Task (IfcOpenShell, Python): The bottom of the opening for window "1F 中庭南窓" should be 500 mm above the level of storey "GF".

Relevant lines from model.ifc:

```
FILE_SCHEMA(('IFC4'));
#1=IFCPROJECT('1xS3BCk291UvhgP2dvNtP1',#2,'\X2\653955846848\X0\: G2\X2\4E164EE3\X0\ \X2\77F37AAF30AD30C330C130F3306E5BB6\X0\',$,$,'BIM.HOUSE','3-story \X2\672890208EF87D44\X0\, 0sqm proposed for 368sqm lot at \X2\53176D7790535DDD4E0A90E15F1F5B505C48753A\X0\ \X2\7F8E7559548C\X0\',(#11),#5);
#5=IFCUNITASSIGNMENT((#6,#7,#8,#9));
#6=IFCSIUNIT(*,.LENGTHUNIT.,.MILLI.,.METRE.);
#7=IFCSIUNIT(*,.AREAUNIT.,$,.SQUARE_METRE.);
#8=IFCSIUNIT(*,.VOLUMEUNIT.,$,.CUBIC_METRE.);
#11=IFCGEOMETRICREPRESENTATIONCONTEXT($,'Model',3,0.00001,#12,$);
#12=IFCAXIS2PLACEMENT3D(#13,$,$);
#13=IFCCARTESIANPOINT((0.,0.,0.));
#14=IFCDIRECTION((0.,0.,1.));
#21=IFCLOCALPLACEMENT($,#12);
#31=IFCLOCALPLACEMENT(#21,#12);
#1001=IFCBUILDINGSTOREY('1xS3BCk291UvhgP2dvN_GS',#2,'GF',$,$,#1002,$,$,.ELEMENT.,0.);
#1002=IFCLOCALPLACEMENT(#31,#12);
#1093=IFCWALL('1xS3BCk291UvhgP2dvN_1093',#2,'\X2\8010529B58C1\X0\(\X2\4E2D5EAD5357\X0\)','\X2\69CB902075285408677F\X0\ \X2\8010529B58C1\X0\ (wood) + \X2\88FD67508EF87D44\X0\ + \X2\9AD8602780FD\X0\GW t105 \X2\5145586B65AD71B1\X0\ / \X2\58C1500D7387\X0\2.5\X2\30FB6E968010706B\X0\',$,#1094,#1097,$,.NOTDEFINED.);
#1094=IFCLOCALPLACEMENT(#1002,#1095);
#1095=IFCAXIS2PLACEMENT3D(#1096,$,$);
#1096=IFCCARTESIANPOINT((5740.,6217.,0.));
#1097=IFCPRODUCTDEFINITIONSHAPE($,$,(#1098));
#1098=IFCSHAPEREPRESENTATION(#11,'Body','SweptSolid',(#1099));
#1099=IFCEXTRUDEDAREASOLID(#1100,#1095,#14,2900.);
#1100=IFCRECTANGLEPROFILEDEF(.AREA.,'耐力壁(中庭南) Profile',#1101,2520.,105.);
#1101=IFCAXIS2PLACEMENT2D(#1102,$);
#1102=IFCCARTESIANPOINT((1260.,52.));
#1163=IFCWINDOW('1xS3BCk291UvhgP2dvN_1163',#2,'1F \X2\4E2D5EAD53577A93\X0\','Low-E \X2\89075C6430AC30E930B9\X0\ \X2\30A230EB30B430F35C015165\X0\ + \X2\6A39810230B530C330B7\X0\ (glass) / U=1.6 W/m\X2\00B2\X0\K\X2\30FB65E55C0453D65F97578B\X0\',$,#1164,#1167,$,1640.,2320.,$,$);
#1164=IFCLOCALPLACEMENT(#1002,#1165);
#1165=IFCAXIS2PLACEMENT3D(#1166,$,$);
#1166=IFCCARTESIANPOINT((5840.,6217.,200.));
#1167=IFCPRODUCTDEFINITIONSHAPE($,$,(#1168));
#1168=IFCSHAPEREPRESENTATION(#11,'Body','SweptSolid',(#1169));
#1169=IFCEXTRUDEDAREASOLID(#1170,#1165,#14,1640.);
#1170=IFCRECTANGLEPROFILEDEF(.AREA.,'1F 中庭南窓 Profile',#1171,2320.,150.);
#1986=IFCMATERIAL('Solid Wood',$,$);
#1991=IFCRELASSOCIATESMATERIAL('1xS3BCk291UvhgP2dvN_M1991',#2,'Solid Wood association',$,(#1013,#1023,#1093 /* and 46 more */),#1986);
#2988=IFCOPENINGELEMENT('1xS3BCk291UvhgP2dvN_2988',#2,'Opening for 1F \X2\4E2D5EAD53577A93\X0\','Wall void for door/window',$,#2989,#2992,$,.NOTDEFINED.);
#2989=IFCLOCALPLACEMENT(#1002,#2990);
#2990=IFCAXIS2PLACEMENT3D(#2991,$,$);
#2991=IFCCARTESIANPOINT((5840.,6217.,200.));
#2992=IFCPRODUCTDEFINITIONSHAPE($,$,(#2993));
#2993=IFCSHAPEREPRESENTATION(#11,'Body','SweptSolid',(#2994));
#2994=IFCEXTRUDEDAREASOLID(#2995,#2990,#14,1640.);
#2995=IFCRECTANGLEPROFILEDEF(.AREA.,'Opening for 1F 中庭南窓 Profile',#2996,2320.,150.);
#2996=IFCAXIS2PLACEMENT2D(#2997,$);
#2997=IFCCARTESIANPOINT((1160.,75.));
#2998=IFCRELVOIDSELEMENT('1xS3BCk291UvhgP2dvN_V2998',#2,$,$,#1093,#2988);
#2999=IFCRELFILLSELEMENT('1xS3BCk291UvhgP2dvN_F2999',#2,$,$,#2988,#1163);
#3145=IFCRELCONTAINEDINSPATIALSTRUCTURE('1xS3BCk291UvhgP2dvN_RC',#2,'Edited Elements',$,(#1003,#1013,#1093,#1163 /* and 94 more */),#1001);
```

```python
import numpy as np
import ifcopenshell
import ifcopenshell.api.geometry
import ifcopenshell.geom
import ifcopenshell.util.element
import ifcopenshell.util.placement
import ifcopenshell.util.shape
import ifcopenshell.util.unit

model = ifcopenshell.open("model.ifc")
unit_scale = ifcopenshell.util.unit.calculate_unit_scale(model)

window = model.by_guid("1xS3BCk291UvhgP2dvN_1163")
opening = window.FillsVoids[0].RelatingOpeningElement
storey = ifcopenshell.util.element.get_container(window, ifc_class="IfcBuildingStorey")
level = ifcopenshell.util.placement.get_local_placement(storey.ObjectPlacement)[2, 3]

# The opening's origin need not be at the sill, so measure its lowest point.
shape = ifcopenshell.geom.create_shape(ifcopenshell.geom.settings(), opening)
bottom = ifcopenshell.util.shape.get_shape_bottom_elevation(shape, shape.geometry) / unit_scale
dz = level + 0.5 / unit_scale - bottom

shift = np.array([0.0, 0.0, dz])
# The window is not placed relative to its opening, so move both.
for product in (opening, window):
    matrix = ifcopenshell.util.placement.get_local_placement(product.ObjectPlacement)
    matrix[:3, 3] += shift
    ifcopenshell.api.geometry.edit_object_placement(model, product=product, matrix=matrix, is_si=False)

print(f"moved by {dz * unit_scale:+.3f} m")

model.write("model_updated.ifc")
```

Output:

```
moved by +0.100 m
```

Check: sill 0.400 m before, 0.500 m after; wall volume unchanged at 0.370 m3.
